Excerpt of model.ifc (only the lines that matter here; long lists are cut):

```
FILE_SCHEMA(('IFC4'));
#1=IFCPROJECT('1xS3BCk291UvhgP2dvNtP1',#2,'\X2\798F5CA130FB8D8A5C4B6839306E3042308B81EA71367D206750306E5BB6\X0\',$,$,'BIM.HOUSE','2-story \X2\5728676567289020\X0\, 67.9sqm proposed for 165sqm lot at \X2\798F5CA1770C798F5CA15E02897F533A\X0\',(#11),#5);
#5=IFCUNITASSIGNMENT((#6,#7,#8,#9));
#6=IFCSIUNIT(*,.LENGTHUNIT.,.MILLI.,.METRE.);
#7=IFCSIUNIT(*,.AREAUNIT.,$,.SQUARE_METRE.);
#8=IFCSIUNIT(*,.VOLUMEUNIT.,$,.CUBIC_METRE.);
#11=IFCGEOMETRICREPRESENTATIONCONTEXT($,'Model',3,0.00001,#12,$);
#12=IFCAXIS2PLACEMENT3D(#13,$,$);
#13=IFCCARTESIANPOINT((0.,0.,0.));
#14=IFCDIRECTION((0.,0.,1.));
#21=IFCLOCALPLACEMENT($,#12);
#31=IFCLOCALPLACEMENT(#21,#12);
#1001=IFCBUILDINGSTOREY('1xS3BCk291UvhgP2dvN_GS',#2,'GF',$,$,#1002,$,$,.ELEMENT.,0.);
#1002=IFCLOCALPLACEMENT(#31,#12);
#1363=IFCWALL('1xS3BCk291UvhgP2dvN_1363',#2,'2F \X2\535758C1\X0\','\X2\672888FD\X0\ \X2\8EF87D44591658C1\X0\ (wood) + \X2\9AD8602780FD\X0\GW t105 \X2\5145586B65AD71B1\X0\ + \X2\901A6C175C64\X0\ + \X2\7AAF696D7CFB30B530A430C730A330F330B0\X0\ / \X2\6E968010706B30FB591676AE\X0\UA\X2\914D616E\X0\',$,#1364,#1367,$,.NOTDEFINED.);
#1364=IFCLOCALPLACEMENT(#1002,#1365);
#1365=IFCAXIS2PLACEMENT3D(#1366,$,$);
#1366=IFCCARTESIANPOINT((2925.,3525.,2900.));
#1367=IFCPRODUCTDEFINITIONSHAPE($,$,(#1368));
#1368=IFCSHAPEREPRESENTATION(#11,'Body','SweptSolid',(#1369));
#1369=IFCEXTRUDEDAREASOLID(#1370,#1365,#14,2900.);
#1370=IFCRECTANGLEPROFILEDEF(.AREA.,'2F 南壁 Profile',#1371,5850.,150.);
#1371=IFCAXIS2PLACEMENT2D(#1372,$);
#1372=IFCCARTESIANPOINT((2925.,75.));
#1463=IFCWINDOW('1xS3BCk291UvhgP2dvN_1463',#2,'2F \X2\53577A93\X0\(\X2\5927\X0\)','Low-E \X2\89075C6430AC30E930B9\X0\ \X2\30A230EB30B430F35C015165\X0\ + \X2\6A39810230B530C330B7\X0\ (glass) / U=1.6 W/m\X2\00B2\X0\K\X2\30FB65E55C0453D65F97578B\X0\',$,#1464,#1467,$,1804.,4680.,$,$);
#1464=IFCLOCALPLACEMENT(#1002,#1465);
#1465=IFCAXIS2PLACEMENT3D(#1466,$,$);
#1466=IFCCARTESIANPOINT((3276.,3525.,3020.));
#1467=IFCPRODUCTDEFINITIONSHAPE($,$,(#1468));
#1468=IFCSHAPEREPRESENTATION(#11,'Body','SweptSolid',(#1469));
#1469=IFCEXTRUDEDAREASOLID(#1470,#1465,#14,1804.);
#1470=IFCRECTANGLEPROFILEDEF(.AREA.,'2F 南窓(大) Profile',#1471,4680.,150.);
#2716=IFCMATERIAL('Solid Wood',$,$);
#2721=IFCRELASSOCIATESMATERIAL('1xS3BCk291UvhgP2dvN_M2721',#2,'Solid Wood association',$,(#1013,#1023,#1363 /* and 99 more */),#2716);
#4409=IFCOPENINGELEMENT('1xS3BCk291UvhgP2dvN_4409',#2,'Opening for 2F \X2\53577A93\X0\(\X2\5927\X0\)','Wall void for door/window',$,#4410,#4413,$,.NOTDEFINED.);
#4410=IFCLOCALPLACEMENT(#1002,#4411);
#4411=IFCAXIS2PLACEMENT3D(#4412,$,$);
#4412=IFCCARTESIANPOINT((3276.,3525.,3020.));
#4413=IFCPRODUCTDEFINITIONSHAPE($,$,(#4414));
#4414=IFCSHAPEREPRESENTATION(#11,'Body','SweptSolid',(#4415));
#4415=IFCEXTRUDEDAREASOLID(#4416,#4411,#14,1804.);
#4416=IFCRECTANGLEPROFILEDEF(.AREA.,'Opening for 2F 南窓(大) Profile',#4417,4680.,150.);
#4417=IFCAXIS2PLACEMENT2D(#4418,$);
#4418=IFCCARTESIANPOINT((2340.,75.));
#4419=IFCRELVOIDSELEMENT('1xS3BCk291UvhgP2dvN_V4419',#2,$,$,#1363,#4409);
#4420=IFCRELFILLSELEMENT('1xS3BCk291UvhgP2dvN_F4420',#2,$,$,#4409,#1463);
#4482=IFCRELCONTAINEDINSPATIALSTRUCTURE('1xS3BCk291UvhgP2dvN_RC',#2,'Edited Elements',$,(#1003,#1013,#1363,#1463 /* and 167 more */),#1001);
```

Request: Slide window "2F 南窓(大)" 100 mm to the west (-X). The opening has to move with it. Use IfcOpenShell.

```python
import ifcopenshell
import ifcopenshell.api.geometry
import ifcopenshell.util.placement
import ifcopenshell.util.unit

model = ifcopenshell.open("model.ifc")
unit_scale = ifcopenshell.util.unit.calculate_unit_scale(model)

window = model.by_guid("1xS3BCk291UvhgP2dvN_1463")
opening = window.FillsVoids[0].RelatingOpeningElement
wall = opening.VoidsElements[0].RelatingBuildingElement

wall_matrix = ifcopenshell.util.placement.get_local_placement(wall.ObjectPlacement)
shift = wall_matrix[:3, 0] * -0.1 / unit_scale
before = ifcopenshell.util.placement.get_local_placement(window.ObjectPlacement)[:3, 3].copy()

# The window is not placed relative to its opening, so move both.
for product in (opening, window):
    matrix = ifcopenshell.util.placement.get_local_placement(product.ObjectPlacement)
    matrix[:3, 3] += shift
    ifcopenshell.api.geometry.edit_object_placement(model, product=product, matrix=matrix, is_si=False)

after = ifcopenshell.util.placement.get_local_placement(window.ObjectPlacement)[:3, 3]
print("window moved by", (after - before).round(3) + 0.0)

model.write("model_edited.ifc")
```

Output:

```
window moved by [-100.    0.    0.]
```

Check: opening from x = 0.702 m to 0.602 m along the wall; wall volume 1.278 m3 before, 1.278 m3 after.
